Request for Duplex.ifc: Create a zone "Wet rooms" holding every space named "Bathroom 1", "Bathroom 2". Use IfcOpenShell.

First a look at what the model holds.

```python
import ifcopenshell

model = ifcopenshell.open("Duplex.ifc")
print(model.schema)
seen = {}
for space in model.by_type("IfcSpace"):
    seen[space.LongName] = seen.get(space.LongName, 0) + 1
for name, count in sorted(seen.items(), key=str):
    print(count, "x", name)
print("zones:", [z.Name for z in model.by_type("IfcZone")][:20])
```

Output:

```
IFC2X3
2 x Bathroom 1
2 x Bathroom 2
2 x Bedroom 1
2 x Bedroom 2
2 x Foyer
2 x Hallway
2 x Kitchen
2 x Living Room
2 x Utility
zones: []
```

```python
import ifcopenshell
import ifcopenshell.api.group
import ifcopenshell.api.root

model = ifcopenshell.open("Duplex.ifc")

names = {"Bathroom 1", "Bathroom 2"}
spaces = [s for s in model.by_type("IfcSpace") if s.LongName in names]

zone = ifcopenshell.api.root.create_entity(model, ifc_class="IfcZone", name="Wet rooms")
ifcopenshell.api.group.assign_group(model, products=spaces, group=zone)
print(len(spaces), "spaces in", zone.Name)

model.write("Duplex_rev.ifc")
```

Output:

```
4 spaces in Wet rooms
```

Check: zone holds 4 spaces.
